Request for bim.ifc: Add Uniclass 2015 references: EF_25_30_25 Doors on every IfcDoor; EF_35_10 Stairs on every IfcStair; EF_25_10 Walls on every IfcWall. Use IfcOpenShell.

First a look at what the model holds.

```python
import ifcopenshell

model = ifcopenshell.open("bim.ifc")
print(model.schema)
print("classifications:", [c.Name for c in model.by_type("IfcClassification")])
for ifc_class in ("IfcDoor", "IfcRoof", "IfcStair", "IfcWall", "IfcWindow"):
    print(ifc_class, len(model.by_type(ifc_class)))
```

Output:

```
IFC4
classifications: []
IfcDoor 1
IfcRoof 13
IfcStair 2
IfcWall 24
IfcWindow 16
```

```python
import ifcopenshell
import ifcopenshell.api.classification

model = ifcopenshell.open("bim.ifc")

system = ifcopenshell.api.classification.add_classification(model, classification="Uniclass 2015")

codes = {
    "IfcDoor": ("EF_25_30_25", "Doors"),
    "IfcStair": ("EF_35_10", "Stairs"),
    "IfcWall": ("EF_25_10", "Walls"),
}
for ifc_class, (code, name) in codes.items():
    products = model.by_type(ifc_class)
    ifcopenshell.api.classification.add_reference(
        model, products=products, classification=system, identification=code, name=name
    )
    print(code, len(products))

model.write("bim-out.ifc")
```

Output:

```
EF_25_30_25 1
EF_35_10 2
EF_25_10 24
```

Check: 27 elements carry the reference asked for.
